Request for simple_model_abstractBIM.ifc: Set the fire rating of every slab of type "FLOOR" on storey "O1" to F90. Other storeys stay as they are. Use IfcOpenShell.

First a look at what the model holds.

```python
import ifcopenshell
import ifcopenshell.util.element

model = ifcopenshell.open("simple_model_abstractBIM.ifc")
print(model.schema)
storey = next(s for s in model.by_type("IfcBuildingStorey") if s.Name == "O1")
slabs = [e for e in ifcopenshell.util.element.get_decomposition(storey) if e.is_a("IfcSlab")]
seen = {}
for e in slabs:
    element_type = ifcopenshell.util.element.get_type(e)
    key = (element_type.Name if element_type != e and element_type else None, ifcopenshell.util.element.get_pset(e, "Pset_SlabCommon", "FireRating"))
    seen[key] = seen.get(key, 0) + 1
for (name, value), count in sorted(seen.items(), key=str):
    print(count, "x", name, "|", value)
```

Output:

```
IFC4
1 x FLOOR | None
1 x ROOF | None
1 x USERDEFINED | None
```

```python
import ifcopenshell
import ifcopenshell.api.pset
import ifcopenshell.util.element

model = ifcopenshell.open("simple_model_abstractBIM.ifc")

storey = next(s for s in model.by_type("IfcBuildingStorey") if s.Name == "O1")
slabs = [e for e in ifcopenshell.util.element.get_decomposition(storey) if e.is_a("IfcSlab")]

count = 0
for e in slabs:
    element_type = ifcopenshell.util.element.get_type(e)
    if element_type in (None, e) or element_type.Name != "FLOOR":
        continue
    # add_pset returns the element's existing set when there is one.
    pset = ifcopenshell.api.pset.add_pset(model, product=e, name="Pset_SlabCommon")
    ifcopenshell.api.pset.edit_pset(model, pset=pset, properties={"FireRating": "F90"})
    count += 1

print(count, "slabs updated")

model.write("simple_model_abstractBIM_v2.ifc")
```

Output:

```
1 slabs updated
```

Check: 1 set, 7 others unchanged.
